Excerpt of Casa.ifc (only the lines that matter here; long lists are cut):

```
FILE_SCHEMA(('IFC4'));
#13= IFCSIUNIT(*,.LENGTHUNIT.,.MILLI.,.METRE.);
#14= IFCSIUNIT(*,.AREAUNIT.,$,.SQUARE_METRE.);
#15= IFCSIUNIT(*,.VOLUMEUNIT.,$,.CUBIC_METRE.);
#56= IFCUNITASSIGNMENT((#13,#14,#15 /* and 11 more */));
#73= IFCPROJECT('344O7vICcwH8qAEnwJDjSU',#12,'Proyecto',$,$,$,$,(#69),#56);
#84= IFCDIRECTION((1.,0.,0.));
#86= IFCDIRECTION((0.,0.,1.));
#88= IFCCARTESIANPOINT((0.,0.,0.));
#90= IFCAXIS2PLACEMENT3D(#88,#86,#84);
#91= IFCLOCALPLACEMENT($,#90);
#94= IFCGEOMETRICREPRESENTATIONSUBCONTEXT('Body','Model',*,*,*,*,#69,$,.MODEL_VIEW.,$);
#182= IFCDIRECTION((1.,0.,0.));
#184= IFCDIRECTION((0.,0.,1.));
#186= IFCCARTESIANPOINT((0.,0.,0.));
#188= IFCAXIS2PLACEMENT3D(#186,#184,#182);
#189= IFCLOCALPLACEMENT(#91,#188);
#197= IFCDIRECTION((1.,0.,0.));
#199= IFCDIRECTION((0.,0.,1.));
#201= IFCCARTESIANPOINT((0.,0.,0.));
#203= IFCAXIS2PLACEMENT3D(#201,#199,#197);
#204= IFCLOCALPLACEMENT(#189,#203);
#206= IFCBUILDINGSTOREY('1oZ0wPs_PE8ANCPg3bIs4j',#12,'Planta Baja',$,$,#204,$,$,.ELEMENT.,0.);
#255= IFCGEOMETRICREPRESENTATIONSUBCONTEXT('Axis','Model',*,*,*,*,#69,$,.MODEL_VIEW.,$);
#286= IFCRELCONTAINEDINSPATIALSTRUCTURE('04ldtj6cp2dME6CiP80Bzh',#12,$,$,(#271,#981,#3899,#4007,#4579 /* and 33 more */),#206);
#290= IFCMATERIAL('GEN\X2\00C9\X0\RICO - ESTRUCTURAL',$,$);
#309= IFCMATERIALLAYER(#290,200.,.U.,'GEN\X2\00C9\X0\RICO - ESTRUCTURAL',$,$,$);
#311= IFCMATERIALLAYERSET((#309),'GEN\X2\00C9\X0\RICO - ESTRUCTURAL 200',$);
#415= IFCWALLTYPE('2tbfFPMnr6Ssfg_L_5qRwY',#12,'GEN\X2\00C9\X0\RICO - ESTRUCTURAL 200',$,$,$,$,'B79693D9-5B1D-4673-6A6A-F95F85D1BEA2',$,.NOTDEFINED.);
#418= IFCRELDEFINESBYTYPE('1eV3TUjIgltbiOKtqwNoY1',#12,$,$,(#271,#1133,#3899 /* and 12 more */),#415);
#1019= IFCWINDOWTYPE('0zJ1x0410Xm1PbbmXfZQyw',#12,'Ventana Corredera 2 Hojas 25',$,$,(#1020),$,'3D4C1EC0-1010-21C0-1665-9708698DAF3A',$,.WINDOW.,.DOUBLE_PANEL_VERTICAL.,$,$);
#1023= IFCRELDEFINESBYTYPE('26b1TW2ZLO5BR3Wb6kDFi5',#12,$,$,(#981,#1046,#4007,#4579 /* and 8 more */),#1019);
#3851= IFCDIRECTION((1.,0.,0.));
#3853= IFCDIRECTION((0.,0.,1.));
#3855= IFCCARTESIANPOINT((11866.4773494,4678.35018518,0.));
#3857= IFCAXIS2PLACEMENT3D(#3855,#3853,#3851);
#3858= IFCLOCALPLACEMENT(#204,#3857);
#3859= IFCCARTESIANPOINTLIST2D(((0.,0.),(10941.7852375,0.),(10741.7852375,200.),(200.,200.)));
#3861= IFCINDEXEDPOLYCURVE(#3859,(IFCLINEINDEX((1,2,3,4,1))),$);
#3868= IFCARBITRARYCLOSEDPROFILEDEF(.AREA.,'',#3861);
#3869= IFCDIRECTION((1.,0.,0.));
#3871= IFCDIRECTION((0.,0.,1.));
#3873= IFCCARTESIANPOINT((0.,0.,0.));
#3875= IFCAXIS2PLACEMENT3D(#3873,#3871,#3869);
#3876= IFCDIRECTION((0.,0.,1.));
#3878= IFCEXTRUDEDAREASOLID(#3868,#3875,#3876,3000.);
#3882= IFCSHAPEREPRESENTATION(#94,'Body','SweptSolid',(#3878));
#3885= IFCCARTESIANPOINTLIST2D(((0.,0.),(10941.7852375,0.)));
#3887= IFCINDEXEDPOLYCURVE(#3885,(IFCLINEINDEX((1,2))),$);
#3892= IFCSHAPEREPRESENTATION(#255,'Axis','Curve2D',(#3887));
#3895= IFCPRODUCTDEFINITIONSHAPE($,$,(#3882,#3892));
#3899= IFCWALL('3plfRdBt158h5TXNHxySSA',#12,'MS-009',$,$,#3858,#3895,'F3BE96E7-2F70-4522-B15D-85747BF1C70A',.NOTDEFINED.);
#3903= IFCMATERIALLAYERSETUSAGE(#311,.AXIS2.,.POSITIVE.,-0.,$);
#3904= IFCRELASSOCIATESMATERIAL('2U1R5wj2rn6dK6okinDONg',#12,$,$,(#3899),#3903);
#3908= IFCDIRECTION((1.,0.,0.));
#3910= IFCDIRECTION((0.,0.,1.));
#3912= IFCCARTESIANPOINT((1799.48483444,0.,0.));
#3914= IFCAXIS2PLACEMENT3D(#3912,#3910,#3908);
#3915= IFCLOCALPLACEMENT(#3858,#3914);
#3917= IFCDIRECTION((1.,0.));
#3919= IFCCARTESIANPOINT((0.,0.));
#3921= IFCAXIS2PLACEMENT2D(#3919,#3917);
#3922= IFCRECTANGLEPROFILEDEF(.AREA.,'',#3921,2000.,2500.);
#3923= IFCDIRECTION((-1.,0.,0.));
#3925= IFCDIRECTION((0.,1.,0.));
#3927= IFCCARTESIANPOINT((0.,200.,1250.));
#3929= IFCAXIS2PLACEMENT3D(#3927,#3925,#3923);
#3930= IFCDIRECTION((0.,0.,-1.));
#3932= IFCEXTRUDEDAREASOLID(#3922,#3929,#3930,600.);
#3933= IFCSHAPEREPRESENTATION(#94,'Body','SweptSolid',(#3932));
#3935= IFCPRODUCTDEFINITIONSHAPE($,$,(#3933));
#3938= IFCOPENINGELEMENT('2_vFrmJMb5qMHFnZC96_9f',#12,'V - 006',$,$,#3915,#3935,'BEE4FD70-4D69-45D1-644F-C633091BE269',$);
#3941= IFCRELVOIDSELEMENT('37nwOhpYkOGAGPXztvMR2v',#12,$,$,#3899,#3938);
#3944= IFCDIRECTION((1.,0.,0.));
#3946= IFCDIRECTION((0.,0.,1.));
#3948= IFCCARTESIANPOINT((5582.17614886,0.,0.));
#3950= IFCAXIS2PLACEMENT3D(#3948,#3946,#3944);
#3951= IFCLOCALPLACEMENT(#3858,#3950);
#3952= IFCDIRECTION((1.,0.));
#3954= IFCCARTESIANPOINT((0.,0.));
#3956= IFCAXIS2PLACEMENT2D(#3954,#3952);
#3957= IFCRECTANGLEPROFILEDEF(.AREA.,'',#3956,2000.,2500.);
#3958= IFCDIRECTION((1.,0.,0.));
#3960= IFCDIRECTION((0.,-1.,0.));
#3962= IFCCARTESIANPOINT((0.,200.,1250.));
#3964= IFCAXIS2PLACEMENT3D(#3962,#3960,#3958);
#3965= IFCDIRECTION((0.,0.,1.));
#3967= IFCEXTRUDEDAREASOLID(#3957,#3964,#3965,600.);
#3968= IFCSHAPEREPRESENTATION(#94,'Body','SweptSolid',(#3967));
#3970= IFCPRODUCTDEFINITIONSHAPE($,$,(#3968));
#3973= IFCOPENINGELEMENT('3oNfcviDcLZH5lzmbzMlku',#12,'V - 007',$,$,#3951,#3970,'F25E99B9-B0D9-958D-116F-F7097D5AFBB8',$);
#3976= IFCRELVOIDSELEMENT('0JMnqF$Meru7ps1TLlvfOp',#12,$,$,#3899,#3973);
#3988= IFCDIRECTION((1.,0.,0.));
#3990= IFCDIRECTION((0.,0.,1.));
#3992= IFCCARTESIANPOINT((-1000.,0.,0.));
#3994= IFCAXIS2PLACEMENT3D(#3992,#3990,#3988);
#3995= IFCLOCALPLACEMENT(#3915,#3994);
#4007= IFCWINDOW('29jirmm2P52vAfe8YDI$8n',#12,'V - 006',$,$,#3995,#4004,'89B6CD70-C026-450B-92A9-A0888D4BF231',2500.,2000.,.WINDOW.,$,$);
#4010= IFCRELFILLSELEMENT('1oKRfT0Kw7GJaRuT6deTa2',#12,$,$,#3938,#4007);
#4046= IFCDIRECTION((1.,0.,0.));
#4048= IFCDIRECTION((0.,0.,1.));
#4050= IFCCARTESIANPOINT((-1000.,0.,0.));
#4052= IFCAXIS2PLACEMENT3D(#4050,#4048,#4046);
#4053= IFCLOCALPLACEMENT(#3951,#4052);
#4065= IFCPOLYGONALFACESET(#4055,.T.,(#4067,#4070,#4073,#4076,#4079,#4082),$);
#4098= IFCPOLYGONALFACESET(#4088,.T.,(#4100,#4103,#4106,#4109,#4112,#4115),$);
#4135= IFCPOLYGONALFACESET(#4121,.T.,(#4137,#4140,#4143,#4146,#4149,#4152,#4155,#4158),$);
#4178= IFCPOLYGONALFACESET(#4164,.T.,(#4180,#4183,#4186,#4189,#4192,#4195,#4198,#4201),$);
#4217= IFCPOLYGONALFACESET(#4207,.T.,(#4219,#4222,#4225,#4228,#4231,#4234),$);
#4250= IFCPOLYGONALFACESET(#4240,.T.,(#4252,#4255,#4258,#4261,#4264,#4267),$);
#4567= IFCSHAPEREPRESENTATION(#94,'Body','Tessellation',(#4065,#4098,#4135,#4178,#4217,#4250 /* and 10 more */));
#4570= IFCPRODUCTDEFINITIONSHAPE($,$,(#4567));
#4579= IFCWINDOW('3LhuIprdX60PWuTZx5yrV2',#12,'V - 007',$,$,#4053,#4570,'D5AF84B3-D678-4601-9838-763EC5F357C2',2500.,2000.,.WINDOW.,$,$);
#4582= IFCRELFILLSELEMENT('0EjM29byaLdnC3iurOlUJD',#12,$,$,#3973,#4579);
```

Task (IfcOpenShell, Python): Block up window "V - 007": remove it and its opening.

```python
import ifcopenshell
import ifcopenshell.api.feature
import ifcopenshell.api.root
import ifcopenshell.geom
import ifcopenshell.util.shape

model = ifcopenshell.open("Casa.ifc")
settings = ifcopenshell.geom.settings()


def volume(element):
    """Net volume in cubic metres, openings subtracted."""
    shape = ifcopenshell.geom.create_shape(settings, element)
    return ifcopenshell.util.shape.get_volume(shape.geometry)


window = model.by_guid("3LhuIprdX60PWuTZx5yrV2")
opening = window.FillsVoids[0].RelatingOpeningElement
wall = opening.VoidsElements[0].RelatingBuildingElement
before = volume(wall)

ifcopenshell.api.root.remove_product(model, product=window)
ifcopenshell.api.feature.remove_feature(model, feature=opening)

after = volume(wall)

print(f"wall volume {before:.3f} -> {after:.3f} m3")

model.write("Casa_edited.ifc")
```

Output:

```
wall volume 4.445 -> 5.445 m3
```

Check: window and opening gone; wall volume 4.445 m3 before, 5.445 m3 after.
